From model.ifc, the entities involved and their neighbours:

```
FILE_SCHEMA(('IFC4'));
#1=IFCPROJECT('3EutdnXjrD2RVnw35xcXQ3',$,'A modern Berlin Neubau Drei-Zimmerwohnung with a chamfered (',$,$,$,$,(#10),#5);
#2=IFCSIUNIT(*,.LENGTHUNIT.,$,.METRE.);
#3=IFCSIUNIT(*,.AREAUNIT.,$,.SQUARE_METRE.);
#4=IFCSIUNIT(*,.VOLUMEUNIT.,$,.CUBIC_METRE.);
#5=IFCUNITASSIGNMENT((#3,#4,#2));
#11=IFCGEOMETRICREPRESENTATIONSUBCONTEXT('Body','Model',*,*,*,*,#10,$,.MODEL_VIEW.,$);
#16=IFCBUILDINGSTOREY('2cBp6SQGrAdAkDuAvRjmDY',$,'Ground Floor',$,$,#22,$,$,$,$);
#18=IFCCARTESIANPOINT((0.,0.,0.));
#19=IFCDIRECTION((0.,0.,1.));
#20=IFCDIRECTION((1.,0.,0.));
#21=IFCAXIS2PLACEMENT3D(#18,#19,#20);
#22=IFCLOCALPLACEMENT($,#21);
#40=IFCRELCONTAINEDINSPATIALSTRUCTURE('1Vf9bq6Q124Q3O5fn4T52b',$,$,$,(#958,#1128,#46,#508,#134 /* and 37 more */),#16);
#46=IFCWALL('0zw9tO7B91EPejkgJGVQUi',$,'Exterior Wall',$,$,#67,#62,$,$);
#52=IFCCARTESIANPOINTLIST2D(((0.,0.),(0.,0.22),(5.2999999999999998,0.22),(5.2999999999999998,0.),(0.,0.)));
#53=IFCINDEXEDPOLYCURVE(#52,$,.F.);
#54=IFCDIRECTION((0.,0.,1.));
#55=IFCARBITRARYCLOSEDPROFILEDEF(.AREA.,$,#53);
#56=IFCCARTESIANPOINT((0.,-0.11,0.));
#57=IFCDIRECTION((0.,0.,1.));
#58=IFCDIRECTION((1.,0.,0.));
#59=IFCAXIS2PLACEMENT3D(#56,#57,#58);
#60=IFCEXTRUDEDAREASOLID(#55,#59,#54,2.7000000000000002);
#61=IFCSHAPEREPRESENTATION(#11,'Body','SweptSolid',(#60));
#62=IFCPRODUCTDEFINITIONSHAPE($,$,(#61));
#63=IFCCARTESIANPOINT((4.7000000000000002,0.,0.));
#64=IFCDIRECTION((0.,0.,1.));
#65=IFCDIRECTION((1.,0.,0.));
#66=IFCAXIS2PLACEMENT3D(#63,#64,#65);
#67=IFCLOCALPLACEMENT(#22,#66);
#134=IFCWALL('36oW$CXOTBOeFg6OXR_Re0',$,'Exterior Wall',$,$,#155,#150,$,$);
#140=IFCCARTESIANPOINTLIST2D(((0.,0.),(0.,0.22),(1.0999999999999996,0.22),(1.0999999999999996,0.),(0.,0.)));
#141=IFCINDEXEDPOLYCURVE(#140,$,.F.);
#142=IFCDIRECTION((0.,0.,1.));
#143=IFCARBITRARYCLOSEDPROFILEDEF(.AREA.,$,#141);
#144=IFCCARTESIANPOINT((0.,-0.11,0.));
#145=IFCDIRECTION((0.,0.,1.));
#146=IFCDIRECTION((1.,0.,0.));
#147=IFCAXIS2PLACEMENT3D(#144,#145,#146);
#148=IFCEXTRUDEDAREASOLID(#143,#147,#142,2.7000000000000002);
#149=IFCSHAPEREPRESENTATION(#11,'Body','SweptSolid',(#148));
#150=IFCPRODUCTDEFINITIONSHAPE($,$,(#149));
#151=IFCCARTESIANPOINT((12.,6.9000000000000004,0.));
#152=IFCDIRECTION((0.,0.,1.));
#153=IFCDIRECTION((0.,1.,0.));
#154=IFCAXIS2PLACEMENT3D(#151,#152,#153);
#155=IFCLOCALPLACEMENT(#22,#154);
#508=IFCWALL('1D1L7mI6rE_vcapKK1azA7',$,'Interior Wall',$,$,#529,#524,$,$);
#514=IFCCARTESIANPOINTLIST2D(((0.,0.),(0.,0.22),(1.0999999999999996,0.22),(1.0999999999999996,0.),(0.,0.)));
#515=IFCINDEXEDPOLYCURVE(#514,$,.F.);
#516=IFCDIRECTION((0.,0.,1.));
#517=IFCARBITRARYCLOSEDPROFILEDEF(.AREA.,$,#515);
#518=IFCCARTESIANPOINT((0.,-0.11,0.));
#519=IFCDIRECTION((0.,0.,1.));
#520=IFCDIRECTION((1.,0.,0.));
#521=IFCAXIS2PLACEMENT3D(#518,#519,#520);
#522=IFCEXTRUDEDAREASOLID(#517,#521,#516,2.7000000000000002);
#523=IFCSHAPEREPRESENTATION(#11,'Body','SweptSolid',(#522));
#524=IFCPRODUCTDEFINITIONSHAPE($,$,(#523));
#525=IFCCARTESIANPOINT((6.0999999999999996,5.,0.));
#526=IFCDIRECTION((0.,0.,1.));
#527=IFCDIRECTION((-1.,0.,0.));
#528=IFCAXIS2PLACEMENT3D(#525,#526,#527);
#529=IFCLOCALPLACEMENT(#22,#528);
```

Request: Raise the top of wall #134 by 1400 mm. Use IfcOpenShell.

```python
import ifcopenshell
import ifcopenshell.geom
import ifcopenshell.util.representation
import ifcopenshell.util.shape
import ifcopenshell.util.unit

model = ifcopenshell.open("model.ifc")
unit_scale = ifcopenshell.util.unit.calculate_unit_scale(model)
settings = ifcopenshell.geom.settings()


def volume(element):
    """Net volume in cubic metres, openings subtracted."""
    shape = ifcopenshell.geom.create_shape(settings, element)
    return ifcopenshell.util.shape.get_volume(shape.geometry)


wall = model.by_guid("36oW$CXOTBOeFg6OXR_Re0")
before = volume(wall)

body = ifcopenshell.util.representation.get_representation(wall, "Model", "Body")
solid = body.Items[0]
old_height = solid.Depth
solid.Depth += 1.4 / unit_scale
after = volume(wall)

print(f"height {old_height:g} -> {solid.Depth:g}, volume {before:.3f} -> {after:.3f} m3")

model.write("model_edited.ifc")
```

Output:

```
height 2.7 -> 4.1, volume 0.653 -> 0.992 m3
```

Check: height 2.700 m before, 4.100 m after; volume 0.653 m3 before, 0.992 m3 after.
